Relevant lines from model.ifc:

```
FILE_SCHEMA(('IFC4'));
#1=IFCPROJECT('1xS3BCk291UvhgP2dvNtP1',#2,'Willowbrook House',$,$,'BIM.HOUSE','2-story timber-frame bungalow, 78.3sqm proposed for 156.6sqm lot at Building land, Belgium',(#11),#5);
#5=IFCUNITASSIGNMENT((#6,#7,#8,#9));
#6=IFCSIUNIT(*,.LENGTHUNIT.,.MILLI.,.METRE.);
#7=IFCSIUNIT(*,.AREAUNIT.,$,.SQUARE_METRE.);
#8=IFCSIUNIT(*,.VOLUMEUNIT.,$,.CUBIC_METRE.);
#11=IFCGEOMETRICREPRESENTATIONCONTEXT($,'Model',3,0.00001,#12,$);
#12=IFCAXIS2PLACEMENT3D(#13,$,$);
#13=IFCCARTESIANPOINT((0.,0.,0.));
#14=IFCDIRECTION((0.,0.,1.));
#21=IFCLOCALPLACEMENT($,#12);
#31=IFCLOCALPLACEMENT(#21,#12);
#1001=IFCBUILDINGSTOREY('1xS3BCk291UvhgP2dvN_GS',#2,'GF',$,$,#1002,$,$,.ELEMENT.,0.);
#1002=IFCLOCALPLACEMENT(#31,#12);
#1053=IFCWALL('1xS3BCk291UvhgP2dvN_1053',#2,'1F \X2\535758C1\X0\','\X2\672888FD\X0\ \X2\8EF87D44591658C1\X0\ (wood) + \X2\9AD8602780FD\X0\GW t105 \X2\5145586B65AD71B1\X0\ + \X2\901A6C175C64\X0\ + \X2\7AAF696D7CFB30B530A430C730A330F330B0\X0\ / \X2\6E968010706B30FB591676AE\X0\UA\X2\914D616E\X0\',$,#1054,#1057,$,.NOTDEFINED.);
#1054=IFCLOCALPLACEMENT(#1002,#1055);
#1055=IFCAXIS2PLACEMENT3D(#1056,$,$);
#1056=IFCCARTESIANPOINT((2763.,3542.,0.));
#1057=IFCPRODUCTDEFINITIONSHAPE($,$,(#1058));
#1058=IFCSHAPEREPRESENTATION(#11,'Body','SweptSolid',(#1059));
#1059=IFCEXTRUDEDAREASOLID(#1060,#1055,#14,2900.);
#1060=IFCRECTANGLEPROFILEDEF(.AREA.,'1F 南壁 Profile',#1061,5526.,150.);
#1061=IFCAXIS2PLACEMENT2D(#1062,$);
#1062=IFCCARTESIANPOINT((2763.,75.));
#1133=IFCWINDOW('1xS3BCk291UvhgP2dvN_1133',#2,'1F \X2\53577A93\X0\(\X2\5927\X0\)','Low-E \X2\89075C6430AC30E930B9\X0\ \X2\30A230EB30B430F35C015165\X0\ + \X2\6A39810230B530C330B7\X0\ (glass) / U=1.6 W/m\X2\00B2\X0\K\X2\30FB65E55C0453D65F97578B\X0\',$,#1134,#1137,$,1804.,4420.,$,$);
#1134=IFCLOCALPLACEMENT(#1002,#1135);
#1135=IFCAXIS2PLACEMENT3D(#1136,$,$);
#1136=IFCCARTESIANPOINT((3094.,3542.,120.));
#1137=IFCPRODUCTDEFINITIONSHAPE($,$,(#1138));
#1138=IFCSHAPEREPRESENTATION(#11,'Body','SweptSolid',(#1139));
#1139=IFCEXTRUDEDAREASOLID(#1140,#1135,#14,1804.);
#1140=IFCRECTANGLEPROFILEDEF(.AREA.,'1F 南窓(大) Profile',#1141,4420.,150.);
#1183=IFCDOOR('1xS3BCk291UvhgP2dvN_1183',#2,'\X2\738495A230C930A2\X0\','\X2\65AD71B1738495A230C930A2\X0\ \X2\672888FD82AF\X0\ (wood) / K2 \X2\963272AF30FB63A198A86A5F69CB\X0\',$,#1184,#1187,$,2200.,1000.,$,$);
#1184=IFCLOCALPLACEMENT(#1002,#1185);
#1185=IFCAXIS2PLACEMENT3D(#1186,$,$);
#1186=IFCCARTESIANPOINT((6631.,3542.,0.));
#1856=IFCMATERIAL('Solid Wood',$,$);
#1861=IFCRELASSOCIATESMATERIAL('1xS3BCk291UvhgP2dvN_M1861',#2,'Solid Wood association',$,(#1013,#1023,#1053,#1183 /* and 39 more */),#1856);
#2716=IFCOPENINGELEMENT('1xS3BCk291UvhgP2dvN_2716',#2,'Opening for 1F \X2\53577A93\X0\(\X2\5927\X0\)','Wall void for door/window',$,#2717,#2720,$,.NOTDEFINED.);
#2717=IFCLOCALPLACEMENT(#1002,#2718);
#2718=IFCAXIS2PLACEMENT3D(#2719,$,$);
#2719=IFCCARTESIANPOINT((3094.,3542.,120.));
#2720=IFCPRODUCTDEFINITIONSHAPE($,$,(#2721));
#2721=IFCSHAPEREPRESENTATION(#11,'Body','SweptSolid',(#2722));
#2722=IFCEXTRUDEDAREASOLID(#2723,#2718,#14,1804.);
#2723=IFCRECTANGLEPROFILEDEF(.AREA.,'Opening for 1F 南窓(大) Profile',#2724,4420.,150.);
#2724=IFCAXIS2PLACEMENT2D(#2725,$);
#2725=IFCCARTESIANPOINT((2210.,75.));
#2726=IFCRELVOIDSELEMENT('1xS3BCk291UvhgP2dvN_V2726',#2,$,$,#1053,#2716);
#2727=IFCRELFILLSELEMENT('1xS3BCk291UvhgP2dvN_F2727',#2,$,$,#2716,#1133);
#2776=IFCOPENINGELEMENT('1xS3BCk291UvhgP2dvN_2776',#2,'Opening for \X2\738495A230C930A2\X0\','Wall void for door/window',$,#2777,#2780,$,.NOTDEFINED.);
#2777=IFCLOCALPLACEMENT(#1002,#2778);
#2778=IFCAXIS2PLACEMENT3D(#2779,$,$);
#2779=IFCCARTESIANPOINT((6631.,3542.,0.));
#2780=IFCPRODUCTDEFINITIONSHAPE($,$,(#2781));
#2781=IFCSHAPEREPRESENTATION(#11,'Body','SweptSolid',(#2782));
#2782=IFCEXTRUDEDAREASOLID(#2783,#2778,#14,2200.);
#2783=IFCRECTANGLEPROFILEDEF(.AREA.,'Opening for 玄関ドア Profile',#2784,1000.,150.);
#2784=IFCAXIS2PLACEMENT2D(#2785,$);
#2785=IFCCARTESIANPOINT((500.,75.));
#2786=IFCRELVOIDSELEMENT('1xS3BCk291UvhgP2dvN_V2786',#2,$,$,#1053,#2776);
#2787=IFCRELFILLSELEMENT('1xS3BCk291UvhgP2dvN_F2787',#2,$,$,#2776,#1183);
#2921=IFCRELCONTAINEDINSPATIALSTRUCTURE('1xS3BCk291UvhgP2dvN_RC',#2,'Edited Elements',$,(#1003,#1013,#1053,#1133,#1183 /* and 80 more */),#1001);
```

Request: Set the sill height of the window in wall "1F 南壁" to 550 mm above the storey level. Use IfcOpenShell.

```python
import numpy as np
import ifcopenshell
import ifcopenshell.api.geometry
import ifcopenshell.geom
import ifcopenshell.util.element
import ifcopenshell.util.placement
import ifcopenshell.util.shape
import ifcopenshell.util.unit

model = ifcopenshell.open("model.ifc")
unit_scale = ifcopenshell.util.unit.calculate_unit_scale(model)

window = model.by_id(1133)
opening = window.FillsVoids[0].RelatingOpeningElement
storey = ifcopenshell.util.element.get_container(window, ifc_class="IfcBuildingStorey")
level = ifcopenshell.util.placement.get_local_placement(storey.ObjectPlacement)[2, 3]

# The opening's origin need not be at the sill, so measure its lowest point.
shape = ifcopenshell.geom.create_shape(ifcopenshell.geom.settings(), opening)
bottom = ifcopenshell.util.shape.get_shape_bottom_elevation(shape, shape.geometry) / unit_scale
dz = level + 0.55 / unit_scale - bottom

shift = np.array([0.0, 0.0, dz])
# The window is not placed relative to its opening, so move both.
for product in (opening, window):
    matrix = ifcopenshell.util.placement.get_local_placement(product.ObjectPlacement)
    matrix[:3, 3] += shift
    ifcopenshell.api.geometry.edit_object_placement(model, product=product, matrix=matrix, is_si=False)

print(f"moved by {dz * unit_scale:+.3f} m")

model.write("model-out.ifc")
```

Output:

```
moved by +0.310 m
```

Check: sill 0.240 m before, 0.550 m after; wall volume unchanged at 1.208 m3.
